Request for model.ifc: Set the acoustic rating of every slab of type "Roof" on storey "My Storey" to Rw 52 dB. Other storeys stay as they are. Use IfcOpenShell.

First a look at what the model holds.

```python
import ifcopenshell
import ifcopenshell.util.element

model = ifcopenshell.open("model.ifc")
print(model.schema)
storey = next(s for s in model.by_type("IfcBuildingStorey") if s.Name == "My Storey")
slabs = [e for e in ifcopenshell.util.element.get_decomposition(storey) if e.is_a("IfcSlab")]
seen = {}
for e in slabs:
    element_type = ifcopenshell.util.element.get_type(e)
    key = (element_type.Name if element_type != e and element_type else None, ifcopenshell.util.element.get_pset(e, "Pset_SlabCommon", "AcousticRating"))
    seen[key] = seen.get(key, 0) + 1
for (name, value), count in sorted(seen.items(), key=str):
    print(count, "x", name, "|", value)
```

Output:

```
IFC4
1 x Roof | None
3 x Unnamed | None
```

```python
import ifcopenshell
import ifcopenshell.api.pset
import ifcopenshell.util.element

model = ifcopenshell.open("model.ifc")

storey = next(s for s in model.by_type("IfcBuildingStorey") if s.Name == "My Storey")
slabs = [e for e in ifcopenshell.util.element.get_decomposition(storey) if e.is_a("IfcSlab")]

count = 0
for e in slabs:
    element_type = ifcopenshell.util.element.get_type(e)
    if element_type in (None, e) or element_type.Name != "Roof":
        continue
    # add_pset returns the element's existing set when there is one.
    pset = ifcopenshell.api.pset.add_pset(model, product=e, name="Pset_SlabCommon")
    ifcopenshell.api.pset.edit_pset(model, pset=pset, properties={"AcousticRating": "Rw 52 dB"})
    count += 1

print(count, "slabs updated")

model.write("model_edited.ifc")
```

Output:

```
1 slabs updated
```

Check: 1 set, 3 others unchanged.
